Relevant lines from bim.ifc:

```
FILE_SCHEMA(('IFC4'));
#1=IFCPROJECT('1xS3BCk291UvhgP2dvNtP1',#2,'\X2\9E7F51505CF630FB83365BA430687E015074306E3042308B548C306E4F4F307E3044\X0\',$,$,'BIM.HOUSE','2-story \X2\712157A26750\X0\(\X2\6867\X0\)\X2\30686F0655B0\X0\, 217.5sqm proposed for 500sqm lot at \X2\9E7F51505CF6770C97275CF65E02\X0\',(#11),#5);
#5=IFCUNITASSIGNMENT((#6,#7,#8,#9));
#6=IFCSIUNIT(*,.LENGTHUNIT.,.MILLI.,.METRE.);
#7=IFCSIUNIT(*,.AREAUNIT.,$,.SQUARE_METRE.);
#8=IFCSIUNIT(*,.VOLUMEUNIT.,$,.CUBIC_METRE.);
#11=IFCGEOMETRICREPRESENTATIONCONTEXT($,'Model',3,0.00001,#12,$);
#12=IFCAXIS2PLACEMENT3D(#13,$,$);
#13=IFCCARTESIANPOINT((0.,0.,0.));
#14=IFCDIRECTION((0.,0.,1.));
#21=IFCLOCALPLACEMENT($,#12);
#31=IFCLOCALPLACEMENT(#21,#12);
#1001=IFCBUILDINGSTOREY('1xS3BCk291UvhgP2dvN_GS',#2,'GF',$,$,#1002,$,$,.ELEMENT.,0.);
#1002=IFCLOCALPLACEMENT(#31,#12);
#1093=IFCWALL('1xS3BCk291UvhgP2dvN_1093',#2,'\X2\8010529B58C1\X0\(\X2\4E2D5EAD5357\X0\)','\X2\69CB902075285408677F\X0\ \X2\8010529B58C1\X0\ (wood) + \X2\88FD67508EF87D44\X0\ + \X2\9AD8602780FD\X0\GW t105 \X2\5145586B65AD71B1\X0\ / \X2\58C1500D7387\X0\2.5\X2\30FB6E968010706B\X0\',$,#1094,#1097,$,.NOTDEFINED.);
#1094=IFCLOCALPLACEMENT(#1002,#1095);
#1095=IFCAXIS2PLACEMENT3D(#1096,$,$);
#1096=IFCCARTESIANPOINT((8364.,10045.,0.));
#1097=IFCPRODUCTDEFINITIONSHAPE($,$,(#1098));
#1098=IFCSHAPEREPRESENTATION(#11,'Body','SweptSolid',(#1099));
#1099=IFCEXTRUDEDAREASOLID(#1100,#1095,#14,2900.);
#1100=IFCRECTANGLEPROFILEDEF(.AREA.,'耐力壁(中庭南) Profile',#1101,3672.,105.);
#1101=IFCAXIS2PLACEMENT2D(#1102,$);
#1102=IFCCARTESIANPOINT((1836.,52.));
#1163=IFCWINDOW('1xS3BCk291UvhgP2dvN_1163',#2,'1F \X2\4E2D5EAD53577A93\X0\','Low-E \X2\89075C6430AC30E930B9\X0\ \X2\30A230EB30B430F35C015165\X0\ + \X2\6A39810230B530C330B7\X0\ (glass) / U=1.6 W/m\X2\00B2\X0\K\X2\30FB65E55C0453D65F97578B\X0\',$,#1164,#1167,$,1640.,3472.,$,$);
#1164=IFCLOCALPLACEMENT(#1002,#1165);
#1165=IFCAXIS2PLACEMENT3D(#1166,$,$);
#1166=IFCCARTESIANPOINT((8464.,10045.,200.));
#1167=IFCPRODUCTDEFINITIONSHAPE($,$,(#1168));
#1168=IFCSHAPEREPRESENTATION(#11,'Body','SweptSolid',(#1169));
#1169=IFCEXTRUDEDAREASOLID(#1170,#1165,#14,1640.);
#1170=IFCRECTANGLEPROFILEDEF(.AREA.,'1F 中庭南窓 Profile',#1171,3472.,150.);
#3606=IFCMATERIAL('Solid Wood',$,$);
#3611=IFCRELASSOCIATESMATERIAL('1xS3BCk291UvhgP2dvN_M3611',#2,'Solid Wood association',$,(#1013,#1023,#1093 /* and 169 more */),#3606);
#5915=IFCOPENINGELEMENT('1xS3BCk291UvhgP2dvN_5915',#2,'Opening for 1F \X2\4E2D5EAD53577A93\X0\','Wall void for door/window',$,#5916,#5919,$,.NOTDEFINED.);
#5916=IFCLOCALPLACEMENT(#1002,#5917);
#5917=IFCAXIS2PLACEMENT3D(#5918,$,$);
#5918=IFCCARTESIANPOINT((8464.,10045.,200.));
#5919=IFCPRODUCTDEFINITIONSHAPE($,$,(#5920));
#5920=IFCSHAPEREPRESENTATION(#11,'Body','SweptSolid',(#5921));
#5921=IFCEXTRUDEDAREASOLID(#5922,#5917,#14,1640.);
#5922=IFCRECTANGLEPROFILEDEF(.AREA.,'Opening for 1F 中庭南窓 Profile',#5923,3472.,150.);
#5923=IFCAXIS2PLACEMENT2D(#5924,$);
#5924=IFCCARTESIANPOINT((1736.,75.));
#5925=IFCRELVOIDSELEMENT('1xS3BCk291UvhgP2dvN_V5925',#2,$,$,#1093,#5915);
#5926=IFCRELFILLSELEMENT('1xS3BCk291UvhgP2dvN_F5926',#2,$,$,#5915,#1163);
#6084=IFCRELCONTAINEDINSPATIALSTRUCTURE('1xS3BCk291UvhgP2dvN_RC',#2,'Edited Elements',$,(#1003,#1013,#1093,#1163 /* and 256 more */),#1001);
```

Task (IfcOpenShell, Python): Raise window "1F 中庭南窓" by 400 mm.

```python
import numpy as np
import ifcopenshell
import ifcopenshell.api.geometry
import ifcopenshell.util.placement
import ifcopenshell.util.unit

model = ifcopenshell.open("bim.ifc")
unit_scale = ifcopenshell.util.unit.calculate_unit_scale(model)

window = model.by_id(1163)
opening = window.FillsVoids[0].RelatingOpeningElement
dz = 400.0

shift = np.array([0.0, 0.0, dz])
# The window is not placed relative to its opening, so move both.
for product in (opening, window):
    matrix = ifcopenshell.util.placement.get_local_placement(product.ObjectPlacement)
    matrix[:3, 3] += shift
    ifcopenshell.api.geometry.edit_object_placement(model, product=product, matrix=matrix, is_si=False)

print(f"moved by {dz * unit_scale:+.3f} m")

model.write("bim_updated.ifc")
```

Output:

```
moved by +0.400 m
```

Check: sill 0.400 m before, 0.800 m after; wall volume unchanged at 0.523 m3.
